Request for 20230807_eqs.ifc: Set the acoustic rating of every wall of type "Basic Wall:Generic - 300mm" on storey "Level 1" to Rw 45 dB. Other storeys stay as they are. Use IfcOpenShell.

First a look at what the model holds.

```python
import ifcopenshell
import ifcopenshell.util.element

model = ifcopenshell.open("20230807_eqs.ifc")
print(model.schema)
storey = next(s for s in model.by_type("IfcBuildingStorey") if s.Name == "Level 1")
walls = [e for e in ifcopenshell.util.element.get_decomposition(storey) if e.is_a("IfcWall")]
seen = {}
for e in walls:
    element_type = ifcopenshell.util.element.get_type(e)
    key = (element_type.Name if element_type != e and element_type else None, ifcopenshell.util.element.get_pset(e, "Pset_WallCommon", "AcousticRating"))
    seen[key] = seen.get(key, 0) + 1
for (name, value), count in sorted(seen.items(), key=str):
    print(count, "x", name, "|", value)
```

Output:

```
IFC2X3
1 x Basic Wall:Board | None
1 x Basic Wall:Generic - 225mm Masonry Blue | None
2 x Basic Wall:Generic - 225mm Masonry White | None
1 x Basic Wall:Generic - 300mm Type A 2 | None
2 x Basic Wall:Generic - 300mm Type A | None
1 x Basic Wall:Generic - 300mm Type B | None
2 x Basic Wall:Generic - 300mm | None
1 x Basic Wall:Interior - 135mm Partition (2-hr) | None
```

```python
import ifcopenshell
import ifcopenshell.api.pset
import ifcopenshell.util.element

model = ifcopenshell.open("20230807_eqs.ifc")

storey = next(s for s in model.by_type("IfcBuildingStorey") if s.Name == "Level 1")
walls = [e for e in ifcopenshell.util.element.get_decomposition(storey) if e.is_a("IfcWall")]

count = 0
for e in walls:
    element_type = ifcopenshell.util.element.get_type(e)
    if element_type in (None, e) or element_type.Name != "Basic Wall:Generic - 300mm":
        continue
    # add_pset returns the element's existing set when there is one.
    pset = ifcopenshell.api.pset.add_pset(model, product=e, name="Pset_WallCommon")
    ifcopenshell.api.pset.edit_pset(model, pset=pset, properties={"AcousticRating": "Rw 45 dB"})
    count += 1

print(count, "walls updated")

model.write("20230807_eqs_edited.ifc")
```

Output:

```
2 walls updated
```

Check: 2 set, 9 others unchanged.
